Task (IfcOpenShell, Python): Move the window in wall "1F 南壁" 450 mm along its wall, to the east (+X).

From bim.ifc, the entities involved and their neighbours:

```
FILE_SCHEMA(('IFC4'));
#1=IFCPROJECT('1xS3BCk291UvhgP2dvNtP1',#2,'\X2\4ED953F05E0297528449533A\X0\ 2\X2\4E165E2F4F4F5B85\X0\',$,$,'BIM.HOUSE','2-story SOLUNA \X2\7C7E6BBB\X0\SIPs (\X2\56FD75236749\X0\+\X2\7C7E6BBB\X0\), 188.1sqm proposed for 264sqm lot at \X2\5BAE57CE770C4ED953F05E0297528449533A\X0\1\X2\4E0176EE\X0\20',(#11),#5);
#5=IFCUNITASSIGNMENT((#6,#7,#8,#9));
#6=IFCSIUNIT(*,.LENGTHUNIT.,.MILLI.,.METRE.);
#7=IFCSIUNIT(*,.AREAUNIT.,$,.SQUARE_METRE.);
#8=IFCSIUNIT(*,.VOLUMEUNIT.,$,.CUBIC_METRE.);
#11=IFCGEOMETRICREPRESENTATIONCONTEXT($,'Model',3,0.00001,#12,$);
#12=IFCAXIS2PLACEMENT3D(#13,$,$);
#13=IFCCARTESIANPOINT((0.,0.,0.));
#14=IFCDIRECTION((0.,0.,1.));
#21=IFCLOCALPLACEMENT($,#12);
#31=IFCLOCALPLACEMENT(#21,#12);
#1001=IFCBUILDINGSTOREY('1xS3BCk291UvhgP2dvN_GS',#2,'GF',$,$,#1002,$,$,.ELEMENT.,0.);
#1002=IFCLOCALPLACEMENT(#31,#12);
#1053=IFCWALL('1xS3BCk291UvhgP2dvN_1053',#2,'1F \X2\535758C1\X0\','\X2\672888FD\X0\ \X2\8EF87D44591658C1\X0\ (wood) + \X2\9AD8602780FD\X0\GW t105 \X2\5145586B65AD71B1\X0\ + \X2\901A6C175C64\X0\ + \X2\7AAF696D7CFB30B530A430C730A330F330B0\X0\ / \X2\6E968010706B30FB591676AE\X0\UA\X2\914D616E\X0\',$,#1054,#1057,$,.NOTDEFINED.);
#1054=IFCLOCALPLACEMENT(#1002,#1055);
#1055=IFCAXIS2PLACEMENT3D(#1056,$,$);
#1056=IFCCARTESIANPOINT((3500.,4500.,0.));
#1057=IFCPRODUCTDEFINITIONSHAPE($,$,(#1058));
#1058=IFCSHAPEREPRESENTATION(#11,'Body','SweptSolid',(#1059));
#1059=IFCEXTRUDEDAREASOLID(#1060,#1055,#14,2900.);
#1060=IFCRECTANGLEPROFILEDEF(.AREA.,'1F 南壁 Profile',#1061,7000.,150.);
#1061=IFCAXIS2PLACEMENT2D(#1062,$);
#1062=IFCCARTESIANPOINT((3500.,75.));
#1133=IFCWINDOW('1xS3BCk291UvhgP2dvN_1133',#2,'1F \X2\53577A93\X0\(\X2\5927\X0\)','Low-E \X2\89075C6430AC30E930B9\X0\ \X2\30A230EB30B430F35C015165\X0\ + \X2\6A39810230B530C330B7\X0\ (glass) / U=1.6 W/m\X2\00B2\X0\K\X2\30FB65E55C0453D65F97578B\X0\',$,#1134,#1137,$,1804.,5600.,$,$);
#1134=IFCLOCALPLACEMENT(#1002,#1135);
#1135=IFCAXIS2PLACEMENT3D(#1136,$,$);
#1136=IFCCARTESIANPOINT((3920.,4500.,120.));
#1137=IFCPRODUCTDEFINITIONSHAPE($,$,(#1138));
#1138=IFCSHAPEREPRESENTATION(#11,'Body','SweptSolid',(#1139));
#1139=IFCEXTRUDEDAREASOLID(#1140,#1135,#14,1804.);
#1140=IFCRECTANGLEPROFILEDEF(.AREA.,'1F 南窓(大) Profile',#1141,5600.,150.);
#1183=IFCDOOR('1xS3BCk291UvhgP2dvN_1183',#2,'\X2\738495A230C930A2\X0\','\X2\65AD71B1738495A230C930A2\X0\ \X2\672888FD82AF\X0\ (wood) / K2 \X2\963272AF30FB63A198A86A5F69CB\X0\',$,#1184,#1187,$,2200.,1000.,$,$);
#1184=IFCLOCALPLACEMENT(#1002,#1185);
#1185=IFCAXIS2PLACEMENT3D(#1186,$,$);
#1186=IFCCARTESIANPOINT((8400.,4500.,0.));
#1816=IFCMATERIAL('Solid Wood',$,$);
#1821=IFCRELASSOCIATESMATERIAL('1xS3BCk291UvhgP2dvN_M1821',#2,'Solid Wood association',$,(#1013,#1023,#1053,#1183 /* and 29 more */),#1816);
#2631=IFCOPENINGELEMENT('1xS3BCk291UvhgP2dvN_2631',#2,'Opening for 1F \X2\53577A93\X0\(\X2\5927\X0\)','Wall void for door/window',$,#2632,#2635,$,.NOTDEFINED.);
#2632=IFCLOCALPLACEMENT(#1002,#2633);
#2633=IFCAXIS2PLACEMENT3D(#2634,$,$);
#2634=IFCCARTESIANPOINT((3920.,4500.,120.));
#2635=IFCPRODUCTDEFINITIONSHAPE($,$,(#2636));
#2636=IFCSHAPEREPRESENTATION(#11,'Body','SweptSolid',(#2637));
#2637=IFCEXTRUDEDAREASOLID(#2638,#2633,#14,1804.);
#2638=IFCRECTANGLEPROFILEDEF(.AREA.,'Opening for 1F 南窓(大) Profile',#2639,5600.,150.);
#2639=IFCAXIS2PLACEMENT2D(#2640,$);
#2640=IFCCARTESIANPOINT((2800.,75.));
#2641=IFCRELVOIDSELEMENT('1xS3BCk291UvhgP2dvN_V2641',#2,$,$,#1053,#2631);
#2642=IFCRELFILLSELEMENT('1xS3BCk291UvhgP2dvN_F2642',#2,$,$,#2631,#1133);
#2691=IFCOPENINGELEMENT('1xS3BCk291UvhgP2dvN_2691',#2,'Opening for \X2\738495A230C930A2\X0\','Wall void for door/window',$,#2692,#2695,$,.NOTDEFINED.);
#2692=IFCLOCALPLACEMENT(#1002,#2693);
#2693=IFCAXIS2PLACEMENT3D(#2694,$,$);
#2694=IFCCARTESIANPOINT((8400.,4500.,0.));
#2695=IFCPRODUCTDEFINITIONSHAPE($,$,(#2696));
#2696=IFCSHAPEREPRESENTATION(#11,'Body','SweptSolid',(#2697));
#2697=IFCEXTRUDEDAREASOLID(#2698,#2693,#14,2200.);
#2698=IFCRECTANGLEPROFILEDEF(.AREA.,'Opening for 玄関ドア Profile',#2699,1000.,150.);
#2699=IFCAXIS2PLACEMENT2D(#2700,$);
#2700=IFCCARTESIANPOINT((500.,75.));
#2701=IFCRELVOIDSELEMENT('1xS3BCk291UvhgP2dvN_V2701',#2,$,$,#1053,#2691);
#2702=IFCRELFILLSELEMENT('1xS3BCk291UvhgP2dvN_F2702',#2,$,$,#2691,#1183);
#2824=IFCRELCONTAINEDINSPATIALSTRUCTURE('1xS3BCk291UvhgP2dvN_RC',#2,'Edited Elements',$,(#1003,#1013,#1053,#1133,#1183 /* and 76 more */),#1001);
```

```python
import ifcopenshell
import ifcopenshell.api.geometry
import ifcopenshell.util.placement

model = ifcopenshell.open("bim.ifc")

window = model.by_id(1133)
opening = window.FillsVoids[0].RelatingOpeningElement
wall = opening.VoidsElements[0].RelatingBuildingElement

wall_matrix = ifcopenshell.util.placement.get_local_placement(wall.ObjectPlacement)
shift = wall_matrix[:3, 0] * 450.0
before = ifcopenshell.util.placement.get_local_placement(window.ObjectPlacement)[:3, 3].copy()

# The window is not placed relative to its opening, so move both.
for product in (opening, window):
    matrix = ifcopenshell.util.placement.get_local_placement(product.ObjectPlacement)
    matrix[:3, 3] += shift
    ifcopenshell.api.geometry.edit_object_placement(model, product=product, matrix=matrix, is_si=False)

after = ifcopenshell.util.placement.get_local_placement(window.ObjectPlacement)[:3, 3]
print("window moved by", (after - before).round(3) + 0.0)

model.write("bim_v2.ifc")
```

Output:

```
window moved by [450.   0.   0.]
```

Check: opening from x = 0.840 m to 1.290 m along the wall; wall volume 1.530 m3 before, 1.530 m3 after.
